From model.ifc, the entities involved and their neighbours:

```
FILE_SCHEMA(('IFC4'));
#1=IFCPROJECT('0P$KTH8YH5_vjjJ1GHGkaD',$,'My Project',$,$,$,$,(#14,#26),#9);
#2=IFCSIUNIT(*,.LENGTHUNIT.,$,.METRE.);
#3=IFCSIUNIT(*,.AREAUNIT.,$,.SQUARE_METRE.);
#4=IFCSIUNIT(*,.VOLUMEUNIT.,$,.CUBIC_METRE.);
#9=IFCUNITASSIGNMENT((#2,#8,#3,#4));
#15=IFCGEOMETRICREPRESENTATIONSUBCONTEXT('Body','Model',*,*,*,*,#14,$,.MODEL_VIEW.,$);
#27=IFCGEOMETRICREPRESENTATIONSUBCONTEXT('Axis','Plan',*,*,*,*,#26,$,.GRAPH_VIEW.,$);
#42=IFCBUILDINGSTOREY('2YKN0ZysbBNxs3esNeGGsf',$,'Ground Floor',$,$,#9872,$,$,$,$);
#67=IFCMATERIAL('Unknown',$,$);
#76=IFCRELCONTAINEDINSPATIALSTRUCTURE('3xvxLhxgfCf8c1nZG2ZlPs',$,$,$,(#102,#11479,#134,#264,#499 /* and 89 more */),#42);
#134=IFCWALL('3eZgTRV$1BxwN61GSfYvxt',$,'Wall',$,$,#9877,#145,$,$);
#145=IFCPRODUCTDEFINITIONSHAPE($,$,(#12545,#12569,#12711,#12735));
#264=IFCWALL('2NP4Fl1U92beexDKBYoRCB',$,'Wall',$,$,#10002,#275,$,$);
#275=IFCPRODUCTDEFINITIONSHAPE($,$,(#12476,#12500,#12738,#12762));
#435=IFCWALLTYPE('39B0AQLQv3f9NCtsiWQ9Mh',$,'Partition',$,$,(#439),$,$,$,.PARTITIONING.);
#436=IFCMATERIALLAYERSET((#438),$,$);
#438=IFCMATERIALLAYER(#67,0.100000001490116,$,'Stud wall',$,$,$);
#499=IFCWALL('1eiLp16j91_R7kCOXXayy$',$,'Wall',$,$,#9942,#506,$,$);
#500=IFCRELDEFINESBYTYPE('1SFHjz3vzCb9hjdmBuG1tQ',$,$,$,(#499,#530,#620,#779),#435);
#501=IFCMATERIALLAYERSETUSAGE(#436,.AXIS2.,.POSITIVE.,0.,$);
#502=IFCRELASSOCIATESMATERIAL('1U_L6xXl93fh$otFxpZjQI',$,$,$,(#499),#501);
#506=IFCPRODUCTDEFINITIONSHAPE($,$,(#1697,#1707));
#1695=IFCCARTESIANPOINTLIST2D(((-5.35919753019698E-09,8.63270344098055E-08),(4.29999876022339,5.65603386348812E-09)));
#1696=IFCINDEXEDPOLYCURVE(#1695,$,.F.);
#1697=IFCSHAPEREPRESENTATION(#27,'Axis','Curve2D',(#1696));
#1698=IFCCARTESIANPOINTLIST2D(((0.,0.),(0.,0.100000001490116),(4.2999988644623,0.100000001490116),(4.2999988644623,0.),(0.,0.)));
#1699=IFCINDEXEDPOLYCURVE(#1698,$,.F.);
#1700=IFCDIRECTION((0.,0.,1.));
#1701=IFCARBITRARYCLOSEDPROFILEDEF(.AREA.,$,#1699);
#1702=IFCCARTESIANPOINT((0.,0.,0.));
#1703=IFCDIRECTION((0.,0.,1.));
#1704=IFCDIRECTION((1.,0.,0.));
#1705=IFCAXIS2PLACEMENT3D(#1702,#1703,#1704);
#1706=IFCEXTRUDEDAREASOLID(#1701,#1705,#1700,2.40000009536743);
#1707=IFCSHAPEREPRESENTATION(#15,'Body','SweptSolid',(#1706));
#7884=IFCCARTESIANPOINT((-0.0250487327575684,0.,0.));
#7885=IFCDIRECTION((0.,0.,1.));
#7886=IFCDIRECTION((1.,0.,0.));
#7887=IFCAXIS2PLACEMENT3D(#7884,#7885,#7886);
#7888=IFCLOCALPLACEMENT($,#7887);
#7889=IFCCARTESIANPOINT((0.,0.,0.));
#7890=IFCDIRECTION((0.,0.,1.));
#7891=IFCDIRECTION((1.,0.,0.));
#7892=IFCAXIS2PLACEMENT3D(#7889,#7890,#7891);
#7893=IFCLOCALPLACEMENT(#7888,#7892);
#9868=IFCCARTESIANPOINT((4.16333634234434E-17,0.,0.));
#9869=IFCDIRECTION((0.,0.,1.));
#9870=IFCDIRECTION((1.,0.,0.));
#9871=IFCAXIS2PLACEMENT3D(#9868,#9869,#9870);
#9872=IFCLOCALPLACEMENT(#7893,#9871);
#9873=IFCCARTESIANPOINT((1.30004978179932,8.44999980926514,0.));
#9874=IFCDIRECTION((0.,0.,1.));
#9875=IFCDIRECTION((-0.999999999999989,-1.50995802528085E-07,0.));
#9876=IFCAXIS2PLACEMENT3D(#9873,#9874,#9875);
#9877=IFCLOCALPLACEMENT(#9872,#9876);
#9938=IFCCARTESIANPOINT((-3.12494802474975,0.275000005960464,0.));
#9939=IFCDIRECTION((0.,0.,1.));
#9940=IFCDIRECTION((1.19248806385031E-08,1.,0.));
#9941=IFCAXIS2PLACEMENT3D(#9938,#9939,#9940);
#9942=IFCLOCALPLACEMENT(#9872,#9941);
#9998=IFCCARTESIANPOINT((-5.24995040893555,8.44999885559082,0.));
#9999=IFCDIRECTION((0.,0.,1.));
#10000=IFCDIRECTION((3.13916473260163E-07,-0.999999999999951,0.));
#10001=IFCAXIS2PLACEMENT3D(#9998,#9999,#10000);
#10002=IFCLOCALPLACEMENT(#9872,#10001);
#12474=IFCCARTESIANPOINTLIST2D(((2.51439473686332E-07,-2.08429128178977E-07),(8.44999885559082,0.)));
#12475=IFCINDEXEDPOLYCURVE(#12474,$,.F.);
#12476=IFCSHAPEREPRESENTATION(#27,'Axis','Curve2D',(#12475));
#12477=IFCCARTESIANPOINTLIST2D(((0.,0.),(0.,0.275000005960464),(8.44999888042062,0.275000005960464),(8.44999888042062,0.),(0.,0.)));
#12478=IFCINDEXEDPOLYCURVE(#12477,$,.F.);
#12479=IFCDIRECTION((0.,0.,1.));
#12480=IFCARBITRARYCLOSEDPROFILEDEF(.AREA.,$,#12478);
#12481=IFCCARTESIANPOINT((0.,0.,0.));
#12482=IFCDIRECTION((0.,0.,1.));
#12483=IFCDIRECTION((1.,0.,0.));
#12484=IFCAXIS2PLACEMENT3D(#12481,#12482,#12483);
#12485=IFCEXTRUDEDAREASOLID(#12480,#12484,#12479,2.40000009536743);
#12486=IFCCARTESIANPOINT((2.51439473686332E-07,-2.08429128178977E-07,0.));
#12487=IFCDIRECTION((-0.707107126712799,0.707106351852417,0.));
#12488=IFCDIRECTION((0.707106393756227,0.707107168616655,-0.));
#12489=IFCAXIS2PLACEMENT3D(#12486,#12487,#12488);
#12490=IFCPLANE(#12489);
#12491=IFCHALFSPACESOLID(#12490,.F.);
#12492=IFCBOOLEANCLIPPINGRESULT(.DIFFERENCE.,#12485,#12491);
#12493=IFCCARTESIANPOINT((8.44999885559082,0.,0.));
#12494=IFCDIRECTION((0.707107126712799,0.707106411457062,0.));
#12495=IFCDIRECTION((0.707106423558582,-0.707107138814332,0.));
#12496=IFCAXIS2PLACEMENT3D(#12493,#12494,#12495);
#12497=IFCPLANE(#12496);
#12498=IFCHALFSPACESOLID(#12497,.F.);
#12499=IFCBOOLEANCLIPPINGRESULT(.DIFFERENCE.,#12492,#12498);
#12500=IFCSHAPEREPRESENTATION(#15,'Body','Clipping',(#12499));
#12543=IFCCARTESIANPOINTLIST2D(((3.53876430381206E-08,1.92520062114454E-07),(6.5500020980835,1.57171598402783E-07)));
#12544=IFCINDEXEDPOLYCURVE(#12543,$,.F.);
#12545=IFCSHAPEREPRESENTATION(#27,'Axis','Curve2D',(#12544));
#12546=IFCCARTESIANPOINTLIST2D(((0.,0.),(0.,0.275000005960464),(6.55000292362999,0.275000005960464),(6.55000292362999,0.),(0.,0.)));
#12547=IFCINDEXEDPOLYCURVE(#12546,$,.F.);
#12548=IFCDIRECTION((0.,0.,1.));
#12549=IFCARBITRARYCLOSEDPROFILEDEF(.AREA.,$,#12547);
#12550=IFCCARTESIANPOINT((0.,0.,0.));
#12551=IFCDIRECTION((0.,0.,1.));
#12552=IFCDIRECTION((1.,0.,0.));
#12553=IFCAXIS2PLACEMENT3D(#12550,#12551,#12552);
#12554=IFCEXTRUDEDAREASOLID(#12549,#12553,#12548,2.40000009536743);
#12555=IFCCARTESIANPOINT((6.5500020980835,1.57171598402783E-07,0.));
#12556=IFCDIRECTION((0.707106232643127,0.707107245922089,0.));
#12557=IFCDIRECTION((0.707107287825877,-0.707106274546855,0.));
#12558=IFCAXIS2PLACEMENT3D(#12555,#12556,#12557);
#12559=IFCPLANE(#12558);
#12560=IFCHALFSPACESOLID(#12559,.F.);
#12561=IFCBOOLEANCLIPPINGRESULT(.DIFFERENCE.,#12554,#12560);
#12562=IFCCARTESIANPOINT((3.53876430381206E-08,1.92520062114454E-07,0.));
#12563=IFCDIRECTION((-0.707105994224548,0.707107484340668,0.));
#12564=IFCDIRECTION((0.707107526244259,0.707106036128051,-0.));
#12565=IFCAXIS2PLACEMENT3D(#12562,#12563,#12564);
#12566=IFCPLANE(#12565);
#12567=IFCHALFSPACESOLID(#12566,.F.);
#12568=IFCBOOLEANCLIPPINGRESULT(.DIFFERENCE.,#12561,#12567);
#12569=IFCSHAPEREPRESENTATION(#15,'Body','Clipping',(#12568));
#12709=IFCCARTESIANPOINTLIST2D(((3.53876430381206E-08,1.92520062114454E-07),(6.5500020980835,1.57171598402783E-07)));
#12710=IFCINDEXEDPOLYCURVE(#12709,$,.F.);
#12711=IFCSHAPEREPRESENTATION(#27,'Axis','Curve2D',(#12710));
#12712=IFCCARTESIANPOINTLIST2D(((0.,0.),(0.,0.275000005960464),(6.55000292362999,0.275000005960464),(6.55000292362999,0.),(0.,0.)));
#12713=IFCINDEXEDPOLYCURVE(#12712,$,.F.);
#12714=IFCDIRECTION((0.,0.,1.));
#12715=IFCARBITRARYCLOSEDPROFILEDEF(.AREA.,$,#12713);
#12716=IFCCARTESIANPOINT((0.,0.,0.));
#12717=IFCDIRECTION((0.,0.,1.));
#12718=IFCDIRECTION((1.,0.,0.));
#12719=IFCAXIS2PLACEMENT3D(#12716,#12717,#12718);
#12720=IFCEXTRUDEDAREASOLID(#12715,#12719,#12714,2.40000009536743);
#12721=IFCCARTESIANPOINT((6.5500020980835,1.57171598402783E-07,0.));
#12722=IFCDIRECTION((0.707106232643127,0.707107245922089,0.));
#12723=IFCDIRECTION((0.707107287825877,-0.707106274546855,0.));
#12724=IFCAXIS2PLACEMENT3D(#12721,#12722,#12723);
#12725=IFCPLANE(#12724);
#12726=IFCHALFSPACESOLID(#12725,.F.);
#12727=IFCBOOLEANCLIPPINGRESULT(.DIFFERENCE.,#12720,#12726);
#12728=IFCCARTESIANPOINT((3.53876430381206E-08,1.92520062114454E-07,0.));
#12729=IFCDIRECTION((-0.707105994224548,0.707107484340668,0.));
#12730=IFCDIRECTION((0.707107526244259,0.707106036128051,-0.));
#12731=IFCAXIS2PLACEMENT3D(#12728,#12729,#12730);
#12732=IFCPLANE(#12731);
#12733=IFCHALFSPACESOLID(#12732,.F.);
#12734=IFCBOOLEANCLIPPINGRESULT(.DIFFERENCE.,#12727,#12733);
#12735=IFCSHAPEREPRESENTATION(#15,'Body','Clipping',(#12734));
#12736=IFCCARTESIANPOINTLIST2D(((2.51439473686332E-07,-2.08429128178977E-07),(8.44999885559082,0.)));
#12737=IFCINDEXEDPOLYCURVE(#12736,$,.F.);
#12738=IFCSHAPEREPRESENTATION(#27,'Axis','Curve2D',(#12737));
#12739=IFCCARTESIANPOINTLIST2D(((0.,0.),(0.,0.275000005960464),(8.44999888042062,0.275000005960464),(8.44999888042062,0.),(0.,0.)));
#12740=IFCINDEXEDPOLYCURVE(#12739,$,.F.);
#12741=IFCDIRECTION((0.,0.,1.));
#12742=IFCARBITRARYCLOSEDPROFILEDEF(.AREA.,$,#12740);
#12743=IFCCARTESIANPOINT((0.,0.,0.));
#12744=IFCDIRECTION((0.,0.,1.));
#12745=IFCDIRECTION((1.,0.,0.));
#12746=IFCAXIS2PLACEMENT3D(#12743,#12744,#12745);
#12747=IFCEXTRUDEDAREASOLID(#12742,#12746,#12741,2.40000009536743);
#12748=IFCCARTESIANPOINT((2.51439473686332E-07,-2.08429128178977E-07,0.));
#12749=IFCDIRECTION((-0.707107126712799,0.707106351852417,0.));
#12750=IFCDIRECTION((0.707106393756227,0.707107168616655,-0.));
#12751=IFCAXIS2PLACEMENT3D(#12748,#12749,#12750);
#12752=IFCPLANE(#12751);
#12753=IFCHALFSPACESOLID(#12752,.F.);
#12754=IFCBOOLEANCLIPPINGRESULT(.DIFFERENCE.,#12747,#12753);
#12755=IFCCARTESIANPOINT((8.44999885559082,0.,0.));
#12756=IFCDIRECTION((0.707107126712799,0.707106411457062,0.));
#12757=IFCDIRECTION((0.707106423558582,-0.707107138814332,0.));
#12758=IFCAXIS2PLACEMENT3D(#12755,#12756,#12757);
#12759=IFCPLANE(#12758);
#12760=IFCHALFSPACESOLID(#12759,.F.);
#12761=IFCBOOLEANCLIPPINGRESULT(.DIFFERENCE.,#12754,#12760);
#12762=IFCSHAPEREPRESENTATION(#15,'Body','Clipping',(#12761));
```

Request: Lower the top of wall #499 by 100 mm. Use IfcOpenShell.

```python
import ifcopenshell
import ifcopenshell.geom
import ifcopenshell.util.representation
import ifcopenshell.util.shape

model = ifcopenshell.open("model.ifc")
settings = ifcopenshell.geom.settings()


def volume(element):
    """Net volume in cubic metres, openings subtracted."""
    shape = ifcopenshell.geom.create_shape(settings, element)
    return ifcopenshell.util.shape.get_volume(shape.geometry)


wall = model.by_guid("1eiLp16j91_R7kCOXXayy$")
before = volume(wall)

body = ifcopenshell.util.representation.get_representation(wall, "Model", "Body")
solid = body.Items[0]
old_height = solid.Depth
solid.Depth -= 0.1
after = volume(wall)

print(f"height {old_height:g} -> {solid.Depth:g}, volume {before:.3f} -> {after:.3f} m3")

model.write("model_updated.ifc")
```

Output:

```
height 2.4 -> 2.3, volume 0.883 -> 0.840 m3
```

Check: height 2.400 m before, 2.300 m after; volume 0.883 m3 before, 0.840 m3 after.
